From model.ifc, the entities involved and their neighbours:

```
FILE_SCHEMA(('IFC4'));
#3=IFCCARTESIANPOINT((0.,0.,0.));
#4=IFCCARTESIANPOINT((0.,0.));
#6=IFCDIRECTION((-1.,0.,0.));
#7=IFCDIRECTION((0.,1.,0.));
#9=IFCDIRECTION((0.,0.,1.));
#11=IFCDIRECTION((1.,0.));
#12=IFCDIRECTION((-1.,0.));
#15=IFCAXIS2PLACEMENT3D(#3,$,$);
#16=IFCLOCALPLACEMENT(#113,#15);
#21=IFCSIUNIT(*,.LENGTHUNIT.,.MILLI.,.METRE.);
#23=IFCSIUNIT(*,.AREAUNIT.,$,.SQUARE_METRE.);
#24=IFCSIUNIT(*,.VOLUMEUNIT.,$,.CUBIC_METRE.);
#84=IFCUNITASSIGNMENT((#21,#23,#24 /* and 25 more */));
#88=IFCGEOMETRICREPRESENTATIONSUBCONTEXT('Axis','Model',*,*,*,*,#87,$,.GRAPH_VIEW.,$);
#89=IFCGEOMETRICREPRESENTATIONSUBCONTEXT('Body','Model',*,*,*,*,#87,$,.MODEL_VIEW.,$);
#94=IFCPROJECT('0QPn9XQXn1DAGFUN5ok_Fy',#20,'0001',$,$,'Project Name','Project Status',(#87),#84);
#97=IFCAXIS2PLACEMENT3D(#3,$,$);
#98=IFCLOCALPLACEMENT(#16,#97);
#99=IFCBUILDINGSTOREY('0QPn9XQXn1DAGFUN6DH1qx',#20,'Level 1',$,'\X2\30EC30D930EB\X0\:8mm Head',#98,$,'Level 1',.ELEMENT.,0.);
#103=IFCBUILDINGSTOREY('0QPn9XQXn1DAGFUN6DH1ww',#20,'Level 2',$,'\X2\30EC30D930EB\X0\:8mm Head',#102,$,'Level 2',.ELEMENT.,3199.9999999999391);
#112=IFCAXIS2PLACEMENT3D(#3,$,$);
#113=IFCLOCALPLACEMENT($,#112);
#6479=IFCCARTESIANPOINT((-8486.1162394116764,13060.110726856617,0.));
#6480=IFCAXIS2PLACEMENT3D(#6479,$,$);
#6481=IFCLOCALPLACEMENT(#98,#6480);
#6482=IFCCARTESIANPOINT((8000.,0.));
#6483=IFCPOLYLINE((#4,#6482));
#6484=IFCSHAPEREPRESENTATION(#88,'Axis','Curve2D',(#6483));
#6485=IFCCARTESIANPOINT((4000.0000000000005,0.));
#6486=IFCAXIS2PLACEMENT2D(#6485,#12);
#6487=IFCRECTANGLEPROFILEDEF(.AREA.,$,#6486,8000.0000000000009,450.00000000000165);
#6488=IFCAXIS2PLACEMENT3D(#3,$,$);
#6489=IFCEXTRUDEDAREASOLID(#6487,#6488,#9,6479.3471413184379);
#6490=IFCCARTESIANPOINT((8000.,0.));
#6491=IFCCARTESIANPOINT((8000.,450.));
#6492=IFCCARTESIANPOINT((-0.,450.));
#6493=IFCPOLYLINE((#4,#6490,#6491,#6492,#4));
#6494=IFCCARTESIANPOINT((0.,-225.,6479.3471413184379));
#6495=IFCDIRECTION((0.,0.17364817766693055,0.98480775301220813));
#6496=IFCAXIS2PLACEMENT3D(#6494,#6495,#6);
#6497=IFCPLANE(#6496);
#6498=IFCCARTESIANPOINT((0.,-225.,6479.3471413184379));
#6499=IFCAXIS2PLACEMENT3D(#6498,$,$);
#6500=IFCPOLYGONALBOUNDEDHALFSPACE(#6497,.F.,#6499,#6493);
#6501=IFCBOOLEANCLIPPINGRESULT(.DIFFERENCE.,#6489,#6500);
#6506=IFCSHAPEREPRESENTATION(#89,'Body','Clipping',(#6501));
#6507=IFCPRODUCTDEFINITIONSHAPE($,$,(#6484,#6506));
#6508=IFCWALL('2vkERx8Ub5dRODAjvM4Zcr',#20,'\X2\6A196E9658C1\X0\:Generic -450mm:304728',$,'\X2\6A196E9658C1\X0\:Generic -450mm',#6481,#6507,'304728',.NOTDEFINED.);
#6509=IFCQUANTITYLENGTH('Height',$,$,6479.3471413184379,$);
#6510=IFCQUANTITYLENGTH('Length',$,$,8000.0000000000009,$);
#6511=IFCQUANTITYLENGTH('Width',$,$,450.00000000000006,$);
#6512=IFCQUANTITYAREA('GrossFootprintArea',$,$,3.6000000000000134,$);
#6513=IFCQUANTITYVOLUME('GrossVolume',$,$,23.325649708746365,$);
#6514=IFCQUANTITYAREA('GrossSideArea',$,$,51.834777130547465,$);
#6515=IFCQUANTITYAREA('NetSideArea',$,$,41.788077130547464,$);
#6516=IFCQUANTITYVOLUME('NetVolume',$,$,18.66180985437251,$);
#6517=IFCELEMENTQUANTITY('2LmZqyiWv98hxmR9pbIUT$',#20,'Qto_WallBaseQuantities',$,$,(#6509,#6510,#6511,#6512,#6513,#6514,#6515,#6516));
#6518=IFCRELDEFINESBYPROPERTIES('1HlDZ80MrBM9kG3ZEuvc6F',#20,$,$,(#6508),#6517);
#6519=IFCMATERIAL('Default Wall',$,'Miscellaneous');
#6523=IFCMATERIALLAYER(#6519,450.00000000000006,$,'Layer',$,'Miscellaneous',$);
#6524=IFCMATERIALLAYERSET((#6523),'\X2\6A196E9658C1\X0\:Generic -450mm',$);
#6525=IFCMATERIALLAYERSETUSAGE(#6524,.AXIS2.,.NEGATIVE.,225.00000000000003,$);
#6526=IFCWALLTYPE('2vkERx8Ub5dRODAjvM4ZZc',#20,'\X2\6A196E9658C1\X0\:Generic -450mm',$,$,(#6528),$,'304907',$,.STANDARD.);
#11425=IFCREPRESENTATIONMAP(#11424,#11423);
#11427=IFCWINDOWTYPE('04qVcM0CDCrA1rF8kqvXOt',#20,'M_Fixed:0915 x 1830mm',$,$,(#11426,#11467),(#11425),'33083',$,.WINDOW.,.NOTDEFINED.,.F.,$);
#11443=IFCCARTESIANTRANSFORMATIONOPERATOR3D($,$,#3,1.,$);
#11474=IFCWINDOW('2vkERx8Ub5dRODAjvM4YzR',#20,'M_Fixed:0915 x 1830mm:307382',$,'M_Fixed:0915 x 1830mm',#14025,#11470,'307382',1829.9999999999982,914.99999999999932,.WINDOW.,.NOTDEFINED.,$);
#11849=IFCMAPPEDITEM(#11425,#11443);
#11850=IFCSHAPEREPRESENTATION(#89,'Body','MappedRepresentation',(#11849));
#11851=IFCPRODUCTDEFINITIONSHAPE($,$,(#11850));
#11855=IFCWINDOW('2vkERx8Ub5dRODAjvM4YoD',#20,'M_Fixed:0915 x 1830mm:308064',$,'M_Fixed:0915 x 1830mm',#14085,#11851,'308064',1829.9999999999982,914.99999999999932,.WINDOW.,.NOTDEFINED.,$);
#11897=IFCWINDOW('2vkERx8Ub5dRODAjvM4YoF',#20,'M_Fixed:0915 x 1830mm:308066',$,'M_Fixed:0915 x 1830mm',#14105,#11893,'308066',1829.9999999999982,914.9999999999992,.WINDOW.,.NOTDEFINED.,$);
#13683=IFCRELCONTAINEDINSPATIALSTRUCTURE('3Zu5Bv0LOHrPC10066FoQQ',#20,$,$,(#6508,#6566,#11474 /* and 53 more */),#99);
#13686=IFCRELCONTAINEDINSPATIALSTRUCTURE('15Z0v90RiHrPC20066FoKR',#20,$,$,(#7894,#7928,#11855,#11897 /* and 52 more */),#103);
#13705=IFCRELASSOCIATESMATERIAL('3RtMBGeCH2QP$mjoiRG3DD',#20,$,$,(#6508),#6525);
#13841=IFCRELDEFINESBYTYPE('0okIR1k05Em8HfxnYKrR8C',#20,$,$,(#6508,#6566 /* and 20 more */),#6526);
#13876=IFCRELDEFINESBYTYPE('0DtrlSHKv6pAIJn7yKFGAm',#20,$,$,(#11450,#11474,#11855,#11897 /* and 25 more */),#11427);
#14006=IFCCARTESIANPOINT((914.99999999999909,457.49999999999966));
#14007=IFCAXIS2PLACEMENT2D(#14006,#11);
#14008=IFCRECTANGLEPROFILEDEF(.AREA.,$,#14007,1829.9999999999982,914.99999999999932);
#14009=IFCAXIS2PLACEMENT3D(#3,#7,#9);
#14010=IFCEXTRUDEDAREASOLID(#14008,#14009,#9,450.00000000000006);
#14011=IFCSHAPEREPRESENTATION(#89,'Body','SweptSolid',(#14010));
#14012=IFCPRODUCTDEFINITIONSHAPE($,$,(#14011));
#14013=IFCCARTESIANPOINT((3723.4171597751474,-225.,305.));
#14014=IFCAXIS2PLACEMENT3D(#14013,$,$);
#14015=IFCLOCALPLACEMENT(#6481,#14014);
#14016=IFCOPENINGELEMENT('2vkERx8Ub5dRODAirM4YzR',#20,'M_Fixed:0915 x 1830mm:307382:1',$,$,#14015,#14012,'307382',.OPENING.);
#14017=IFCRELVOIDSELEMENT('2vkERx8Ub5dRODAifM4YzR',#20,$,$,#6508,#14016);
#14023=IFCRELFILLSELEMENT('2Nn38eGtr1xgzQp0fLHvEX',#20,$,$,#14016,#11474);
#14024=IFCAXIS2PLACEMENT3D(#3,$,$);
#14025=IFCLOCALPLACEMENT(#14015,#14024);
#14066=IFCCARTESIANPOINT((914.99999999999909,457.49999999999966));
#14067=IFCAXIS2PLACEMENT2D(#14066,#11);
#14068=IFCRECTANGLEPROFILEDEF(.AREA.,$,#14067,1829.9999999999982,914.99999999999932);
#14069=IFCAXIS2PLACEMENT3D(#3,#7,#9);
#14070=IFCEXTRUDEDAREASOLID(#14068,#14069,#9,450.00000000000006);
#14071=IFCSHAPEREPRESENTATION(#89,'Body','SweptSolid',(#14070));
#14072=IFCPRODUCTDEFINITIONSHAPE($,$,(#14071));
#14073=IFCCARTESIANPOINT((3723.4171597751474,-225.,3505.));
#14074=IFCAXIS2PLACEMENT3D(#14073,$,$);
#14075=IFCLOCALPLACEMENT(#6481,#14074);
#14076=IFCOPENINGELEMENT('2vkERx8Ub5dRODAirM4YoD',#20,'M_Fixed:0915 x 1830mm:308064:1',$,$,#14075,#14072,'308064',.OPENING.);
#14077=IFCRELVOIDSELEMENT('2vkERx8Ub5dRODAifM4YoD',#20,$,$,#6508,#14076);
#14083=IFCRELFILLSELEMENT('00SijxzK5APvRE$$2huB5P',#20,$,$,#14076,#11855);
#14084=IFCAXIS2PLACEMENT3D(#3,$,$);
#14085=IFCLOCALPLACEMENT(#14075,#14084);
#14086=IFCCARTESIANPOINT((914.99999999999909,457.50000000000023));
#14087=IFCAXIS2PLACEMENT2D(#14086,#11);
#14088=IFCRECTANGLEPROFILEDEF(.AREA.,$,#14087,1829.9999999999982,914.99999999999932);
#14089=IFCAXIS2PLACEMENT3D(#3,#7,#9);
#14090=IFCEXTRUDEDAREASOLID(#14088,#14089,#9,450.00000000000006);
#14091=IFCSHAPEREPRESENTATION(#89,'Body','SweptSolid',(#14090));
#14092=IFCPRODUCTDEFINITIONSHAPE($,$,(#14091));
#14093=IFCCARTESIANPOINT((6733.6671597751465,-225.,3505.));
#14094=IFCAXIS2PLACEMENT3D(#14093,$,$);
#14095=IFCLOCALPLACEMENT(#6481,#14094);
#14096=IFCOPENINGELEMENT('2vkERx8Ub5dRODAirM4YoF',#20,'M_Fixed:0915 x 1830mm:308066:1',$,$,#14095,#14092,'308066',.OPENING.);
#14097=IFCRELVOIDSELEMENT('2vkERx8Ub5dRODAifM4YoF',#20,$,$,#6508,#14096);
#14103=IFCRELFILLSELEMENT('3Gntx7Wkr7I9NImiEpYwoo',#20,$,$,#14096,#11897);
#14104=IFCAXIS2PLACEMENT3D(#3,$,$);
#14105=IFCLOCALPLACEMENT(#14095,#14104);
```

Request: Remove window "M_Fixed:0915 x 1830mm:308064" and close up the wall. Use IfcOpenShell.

```python
import ifcopenshell
import ifcopenshell.api.feature
import ifcopenshell.api.pset
import ifcopenshell.api.root
import ifcopenshell.geom
import ifcopenshell.util.element
import ifcopenshell.util.shape
import ifcopenshell.util.unit

model = ifcopenshell.open("model.ifc")
area_scale = ifcopenshell.util.unit.calculate_unit_scale(model, "AREAUNIT")
volume_scale = ifcopenshell.util.unit.calculate_unit_scale(model, "VOLUMEUNIT")
settings = ifcopenshell.geom.settings()


def volume(element):
    """Net volume in cubic metres, openings subtracted."""
    shape = ifcopenshell.geom.create_shape(settings, element)
    return ifcopenshell.util.shape.get_volume(shape.geometry)


window = model.by_id(11855)
opening = window.FillsVoids[0].RelatingOpeningElement
wall = opening.VoidsElements[0].RelatingBuildingElement
before = volume(wall)

ifcopenshell.api.root.remove_product(model, product=window)
ifcopenshell.api.feature.remove_feature(model, feature=opening)

after = volume(wall)
thickness = 0.45  # wall thickness in metres

# Update the wall's stored quantities.
qto = model.by_id(ifcopenshell.util.element.get_pset(wall, "Qto_WallBaseQuantities", should_inherit=False)["id"])
ifcopenshell.api.pset.edit_qto(model, qto=qto, properties={
    "NetSideArea": after / thickness / area_scale,
    "NetVolume": after / volume_scale,
})

print(f"wall volume {before:.3f} -> {after:.3f} m3")

model.write("model-out.ifc")
```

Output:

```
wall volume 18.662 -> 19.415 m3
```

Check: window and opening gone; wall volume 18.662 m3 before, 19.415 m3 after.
